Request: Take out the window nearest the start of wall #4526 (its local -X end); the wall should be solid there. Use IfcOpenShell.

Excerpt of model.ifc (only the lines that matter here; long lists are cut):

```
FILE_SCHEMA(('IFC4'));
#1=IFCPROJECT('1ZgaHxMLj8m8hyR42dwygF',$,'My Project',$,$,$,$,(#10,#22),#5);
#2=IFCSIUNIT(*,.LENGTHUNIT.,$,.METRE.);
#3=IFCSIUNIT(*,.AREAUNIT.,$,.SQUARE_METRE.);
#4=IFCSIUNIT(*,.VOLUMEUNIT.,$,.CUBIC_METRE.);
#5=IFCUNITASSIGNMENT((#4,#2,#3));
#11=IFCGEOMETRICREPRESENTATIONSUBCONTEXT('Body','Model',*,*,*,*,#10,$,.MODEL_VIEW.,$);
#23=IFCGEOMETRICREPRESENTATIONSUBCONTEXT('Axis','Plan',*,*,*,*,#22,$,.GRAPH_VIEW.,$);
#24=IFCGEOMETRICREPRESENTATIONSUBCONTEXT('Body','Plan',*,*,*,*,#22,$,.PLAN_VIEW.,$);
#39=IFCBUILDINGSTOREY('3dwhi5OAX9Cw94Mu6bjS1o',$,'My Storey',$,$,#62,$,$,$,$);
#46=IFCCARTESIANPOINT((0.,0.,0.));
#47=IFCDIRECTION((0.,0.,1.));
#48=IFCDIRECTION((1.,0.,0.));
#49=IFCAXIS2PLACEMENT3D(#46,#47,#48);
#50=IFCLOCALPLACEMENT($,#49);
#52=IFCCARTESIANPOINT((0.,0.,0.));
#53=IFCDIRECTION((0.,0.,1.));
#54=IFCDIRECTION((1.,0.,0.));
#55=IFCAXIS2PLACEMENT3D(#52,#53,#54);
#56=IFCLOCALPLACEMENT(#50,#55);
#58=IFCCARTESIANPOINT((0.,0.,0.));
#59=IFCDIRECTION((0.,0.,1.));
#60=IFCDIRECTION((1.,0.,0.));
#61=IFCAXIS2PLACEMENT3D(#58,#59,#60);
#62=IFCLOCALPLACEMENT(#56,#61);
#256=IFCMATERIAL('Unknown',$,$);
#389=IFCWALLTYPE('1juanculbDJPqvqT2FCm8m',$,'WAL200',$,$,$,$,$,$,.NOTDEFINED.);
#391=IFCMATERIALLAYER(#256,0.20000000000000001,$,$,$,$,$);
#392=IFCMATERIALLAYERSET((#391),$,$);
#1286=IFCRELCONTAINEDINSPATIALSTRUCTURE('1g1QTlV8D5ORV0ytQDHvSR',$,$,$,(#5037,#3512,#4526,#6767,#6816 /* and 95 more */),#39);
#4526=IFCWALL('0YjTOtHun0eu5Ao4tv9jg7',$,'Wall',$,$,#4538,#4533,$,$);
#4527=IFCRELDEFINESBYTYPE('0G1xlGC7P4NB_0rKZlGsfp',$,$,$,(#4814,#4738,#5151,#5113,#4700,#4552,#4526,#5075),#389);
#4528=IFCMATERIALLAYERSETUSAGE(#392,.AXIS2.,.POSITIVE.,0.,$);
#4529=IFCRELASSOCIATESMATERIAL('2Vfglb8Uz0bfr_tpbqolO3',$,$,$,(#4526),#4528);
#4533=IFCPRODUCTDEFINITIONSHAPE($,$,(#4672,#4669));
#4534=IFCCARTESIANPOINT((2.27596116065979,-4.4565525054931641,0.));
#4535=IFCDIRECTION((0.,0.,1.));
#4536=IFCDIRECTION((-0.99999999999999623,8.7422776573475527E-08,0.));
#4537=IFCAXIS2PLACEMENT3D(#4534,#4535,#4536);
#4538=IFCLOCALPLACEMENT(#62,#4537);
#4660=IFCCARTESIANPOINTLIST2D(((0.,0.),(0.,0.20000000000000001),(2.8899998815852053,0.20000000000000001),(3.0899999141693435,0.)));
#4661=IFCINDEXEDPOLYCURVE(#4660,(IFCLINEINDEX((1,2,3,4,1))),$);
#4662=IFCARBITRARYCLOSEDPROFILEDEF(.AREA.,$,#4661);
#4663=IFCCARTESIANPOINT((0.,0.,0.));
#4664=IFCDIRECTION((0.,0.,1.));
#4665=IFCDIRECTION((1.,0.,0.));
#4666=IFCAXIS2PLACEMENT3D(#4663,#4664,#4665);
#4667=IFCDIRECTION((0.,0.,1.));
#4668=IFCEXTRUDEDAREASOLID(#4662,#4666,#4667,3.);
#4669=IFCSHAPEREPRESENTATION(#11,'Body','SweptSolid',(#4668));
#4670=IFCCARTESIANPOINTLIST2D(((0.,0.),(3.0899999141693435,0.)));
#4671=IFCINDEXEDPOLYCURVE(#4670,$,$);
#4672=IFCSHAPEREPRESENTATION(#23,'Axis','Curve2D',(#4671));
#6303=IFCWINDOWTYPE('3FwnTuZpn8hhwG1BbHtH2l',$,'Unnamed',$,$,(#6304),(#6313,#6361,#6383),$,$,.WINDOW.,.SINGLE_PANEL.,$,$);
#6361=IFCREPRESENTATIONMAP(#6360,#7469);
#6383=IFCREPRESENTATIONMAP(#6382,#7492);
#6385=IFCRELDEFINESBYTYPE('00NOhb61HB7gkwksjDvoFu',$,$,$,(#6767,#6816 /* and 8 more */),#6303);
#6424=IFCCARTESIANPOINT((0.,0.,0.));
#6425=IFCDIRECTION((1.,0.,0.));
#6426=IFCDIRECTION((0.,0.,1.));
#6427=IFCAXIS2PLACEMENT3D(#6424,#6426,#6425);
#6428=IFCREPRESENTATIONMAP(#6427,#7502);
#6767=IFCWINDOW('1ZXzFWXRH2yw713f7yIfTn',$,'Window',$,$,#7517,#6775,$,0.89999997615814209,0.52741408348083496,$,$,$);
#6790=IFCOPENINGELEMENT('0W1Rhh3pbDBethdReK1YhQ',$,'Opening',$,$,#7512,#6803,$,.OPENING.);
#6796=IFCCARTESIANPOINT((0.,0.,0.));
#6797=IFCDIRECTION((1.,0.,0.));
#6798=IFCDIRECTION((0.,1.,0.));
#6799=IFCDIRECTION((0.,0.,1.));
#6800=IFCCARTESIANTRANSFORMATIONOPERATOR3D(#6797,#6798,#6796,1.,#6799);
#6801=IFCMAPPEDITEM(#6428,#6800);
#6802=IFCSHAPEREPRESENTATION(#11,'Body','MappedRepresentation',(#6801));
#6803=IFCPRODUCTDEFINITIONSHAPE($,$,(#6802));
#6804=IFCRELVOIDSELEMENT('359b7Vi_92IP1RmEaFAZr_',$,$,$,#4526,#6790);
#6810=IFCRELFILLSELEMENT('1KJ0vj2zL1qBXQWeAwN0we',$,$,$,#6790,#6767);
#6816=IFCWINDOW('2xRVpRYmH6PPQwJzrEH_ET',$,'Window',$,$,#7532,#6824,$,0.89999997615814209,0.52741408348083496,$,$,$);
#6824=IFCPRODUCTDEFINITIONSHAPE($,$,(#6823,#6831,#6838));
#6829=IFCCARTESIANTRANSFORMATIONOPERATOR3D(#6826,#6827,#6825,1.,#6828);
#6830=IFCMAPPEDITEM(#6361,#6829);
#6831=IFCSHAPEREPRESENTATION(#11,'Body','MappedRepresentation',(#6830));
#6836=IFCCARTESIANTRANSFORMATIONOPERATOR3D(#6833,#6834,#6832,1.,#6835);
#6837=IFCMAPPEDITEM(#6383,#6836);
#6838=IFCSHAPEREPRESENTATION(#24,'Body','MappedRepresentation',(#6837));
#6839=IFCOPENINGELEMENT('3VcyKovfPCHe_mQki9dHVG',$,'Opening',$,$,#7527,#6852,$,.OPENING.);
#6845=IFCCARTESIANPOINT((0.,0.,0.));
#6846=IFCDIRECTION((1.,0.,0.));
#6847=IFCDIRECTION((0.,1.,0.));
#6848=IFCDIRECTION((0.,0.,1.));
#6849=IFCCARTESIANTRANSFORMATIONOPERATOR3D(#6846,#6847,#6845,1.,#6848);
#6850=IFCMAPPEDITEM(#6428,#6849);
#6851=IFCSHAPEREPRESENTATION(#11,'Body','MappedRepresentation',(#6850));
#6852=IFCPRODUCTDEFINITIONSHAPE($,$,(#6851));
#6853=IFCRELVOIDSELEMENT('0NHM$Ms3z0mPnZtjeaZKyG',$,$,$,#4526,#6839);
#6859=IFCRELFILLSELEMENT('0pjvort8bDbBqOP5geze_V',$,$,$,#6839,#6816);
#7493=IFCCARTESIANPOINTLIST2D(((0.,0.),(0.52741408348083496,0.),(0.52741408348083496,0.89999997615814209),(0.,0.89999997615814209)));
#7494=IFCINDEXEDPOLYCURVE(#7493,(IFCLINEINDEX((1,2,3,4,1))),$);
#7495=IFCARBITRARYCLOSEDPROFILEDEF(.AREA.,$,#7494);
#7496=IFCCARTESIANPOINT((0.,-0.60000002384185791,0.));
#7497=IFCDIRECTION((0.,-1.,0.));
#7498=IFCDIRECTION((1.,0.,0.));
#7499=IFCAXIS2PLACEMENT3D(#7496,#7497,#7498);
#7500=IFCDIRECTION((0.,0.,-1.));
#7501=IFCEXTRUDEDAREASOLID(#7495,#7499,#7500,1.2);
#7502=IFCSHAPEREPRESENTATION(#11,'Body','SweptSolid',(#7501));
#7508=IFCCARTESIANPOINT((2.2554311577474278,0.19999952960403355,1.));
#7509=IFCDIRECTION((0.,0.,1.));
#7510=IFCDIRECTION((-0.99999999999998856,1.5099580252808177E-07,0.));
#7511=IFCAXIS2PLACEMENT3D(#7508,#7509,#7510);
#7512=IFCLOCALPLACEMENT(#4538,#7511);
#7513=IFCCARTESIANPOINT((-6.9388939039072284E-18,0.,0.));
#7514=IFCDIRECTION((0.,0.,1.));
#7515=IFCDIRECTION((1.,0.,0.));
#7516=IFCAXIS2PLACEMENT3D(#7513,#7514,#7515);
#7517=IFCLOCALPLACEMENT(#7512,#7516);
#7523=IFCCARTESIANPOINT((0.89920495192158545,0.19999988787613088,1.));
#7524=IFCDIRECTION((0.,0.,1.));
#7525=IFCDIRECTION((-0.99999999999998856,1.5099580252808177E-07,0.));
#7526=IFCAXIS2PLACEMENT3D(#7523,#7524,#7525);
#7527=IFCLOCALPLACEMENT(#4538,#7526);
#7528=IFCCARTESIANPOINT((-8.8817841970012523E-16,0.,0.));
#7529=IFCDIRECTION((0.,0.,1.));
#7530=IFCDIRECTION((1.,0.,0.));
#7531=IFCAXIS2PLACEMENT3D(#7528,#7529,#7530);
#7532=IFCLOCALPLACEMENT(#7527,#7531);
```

```python
import ifcopenshell
import ifcopenshell.api.feature
import ifcopenshell.api.root
import ifcopenshell.geom
import ifcopenshell.util.shape

model = ifcopenshell.open("model.ifc")
settings = ifcopenshell.geom.settings()


def volume(element):
    """Net volume in cubic metres, openings subtracted."""
    shape = ifcopenshell.geom.create_shape(settings, element)
    return ifcopenshell.util.shape.get_volume(shape.geometry)


window = model.by_guid("2xRVpRYmH6PPQwJzrEH_ET")
opening = window.FillsVoids[0].RelatingOpeningElement
wall = opening.VoidsElements[0].RelatingBuildingElement
before = volume(wall)

ifcopenshell.api.root.remove_product(model, product=window)
ifcopenshell.api.feature.remove_feature(model, feature=opening)

after = volume(wall)

print(f"wall volume {before:.3f} -> {after:.3f} m3")

model.write("model_updated.ifc")
```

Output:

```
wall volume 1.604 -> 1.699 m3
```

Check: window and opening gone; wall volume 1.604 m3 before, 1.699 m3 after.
